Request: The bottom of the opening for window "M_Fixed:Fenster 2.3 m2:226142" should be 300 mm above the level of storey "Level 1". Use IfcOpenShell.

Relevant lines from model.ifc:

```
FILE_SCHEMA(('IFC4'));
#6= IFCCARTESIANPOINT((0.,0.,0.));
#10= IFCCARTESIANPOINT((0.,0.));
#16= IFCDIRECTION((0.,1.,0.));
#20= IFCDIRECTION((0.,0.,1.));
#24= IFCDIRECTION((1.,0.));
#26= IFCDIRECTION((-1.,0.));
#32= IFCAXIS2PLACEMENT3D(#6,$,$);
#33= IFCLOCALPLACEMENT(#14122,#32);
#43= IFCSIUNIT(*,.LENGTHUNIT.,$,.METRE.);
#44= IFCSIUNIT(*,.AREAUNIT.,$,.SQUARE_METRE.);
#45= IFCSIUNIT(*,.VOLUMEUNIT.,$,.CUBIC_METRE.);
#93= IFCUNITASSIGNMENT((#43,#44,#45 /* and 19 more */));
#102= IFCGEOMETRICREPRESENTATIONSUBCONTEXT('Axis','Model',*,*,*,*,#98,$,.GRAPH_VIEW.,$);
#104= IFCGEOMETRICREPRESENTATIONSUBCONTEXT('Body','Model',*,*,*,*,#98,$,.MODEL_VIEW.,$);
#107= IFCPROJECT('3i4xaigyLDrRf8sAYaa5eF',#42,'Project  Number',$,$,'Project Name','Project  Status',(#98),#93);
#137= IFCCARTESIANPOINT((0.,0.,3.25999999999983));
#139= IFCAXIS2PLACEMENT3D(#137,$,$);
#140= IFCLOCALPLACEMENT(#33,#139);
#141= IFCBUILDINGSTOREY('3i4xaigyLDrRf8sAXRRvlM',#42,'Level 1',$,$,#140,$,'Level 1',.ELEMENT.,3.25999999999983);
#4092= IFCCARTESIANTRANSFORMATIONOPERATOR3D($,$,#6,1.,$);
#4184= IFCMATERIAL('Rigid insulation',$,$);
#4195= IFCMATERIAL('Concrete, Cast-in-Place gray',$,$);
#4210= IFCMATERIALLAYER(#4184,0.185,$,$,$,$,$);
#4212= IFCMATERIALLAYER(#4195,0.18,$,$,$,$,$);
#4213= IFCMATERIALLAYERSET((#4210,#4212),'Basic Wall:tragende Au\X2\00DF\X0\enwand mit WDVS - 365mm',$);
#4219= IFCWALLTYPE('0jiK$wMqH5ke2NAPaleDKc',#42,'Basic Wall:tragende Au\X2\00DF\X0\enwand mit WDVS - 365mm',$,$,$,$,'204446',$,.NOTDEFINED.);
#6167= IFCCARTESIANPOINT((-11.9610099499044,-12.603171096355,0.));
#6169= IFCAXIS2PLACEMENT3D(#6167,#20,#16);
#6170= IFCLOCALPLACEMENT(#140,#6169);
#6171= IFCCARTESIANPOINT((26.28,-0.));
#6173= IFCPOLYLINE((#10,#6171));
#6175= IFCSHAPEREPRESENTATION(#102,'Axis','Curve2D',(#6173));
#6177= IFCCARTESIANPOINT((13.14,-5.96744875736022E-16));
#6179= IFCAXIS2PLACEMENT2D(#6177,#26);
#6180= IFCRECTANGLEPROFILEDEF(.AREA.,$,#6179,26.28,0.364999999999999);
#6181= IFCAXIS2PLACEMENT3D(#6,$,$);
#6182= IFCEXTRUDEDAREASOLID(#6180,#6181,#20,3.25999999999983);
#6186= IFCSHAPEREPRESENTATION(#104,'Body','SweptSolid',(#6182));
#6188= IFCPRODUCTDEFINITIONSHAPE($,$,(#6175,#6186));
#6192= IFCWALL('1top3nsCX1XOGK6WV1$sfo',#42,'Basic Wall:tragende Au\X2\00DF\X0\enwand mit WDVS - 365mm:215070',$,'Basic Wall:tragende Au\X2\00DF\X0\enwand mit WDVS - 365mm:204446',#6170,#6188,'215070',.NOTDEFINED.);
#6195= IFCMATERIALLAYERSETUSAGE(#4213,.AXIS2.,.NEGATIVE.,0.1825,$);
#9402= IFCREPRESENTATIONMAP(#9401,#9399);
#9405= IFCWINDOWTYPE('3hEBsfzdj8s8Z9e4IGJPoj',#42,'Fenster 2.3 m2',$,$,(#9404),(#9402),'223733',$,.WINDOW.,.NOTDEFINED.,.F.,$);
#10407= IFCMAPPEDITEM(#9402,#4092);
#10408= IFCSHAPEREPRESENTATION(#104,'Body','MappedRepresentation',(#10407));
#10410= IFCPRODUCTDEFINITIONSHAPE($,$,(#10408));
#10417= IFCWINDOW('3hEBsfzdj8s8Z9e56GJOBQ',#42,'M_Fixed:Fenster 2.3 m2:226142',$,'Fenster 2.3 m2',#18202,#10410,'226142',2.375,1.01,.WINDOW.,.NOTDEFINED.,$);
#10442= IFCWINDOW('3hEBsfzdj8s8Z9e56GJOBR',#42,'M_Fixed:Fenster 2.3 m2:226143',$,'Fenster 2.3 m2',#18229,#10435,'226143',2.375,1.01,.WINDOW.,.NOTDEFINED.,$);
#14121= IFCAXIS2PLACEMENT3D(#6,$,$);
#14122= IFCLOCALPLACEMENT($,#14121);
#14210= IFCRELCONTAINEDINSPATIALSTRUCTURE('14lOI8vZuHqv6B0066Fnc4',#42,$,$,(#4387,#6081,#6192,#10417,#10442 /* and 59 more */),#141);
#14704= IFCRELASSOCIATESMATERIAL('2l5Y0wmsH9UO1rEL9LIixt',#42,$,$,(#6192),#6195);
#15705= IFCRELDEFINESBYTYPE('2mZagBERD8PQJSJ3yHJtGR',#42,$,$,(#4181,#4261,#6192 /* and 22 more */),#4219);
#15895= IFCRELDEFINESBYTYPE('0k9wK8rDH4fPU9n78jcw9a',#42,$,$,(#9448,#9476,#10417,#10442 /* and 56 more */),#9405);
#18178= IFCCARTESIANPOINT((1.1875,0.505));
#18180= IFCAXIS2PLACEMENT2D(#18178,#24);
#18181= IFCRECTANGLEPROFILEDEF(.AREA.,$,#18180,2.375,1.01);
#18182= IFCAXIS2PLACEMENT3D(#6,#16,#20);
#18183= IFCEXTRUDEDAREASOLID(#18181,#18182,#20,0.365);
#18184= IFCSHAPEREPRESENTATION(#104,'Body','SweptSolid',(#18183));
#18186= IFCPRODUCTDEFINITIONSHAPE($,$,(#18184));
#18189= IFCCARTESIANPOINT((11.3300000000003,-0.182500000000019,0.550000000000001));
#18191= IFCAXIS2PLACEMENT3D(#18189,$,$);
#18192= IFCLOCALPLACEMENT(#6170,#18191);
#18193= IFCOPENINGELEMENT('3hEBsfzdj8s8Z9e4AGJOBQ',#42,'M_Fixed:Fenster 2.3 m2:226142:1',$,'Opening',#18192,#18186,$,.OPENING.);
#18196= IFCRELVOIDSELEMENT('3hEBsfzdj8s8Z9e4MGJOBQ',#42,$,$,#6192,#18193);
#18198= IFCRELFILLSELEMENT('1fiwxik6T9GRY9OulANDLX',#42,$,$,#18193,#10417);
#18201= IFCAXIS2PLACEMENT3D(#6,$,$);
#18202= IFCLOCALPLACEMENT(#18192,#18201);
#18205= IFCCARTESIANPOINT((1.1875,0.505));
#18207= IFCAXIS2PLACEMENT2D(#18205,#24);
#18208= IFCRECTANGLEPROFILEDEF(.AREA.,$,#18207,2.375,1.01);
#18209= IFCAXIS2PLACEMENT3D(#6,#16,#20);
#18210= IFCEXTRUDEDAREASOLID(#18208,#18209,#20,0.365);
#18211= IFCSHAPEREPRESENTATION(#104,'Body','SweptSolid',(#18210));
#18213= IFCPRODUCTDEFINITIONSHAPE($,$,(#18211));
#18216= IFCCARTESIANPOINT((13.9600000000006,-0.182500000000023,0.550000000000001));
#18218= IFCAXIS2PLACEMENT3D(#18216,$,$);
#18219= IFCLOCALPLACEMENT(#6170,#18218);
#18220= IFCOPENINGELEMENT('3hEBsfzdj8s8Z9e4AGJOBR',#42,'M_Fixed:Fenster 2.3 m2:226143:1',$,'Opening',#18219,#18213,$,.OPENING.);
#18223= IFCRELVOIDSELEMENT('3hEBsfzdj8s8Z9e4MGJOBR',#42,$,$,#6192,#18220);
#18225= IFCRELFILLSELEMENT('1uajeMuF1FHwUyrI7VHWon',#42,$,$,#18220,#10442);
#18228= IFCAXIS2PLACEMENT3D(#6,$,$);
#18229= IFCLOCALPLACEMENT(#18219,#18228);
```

```python
import numpy as np
import ifcopenshell
import ifcopenshell.api.geometry
import ifcopenshell.geom
import ifcopenshell.util.element
import ifcopenshell.util.placement
import ifcopenshell.util.shape
import ifcopenshell.util.unit

model = ifcopenshell.open("model.ifc")
unit_scale = ifcopenshell.util.unit.calculate_unit_scale(model)

window = model.by_guid("3hEBsfzdj8s8Z9e56GJOBQ")
opening = window.FillsVoids[0].RelatingOpeningElement
storey = ifcopenshell.util.element.get_container(window, ifc_class="IfcBuildingStorey")
level = ifcopenshell.util.placement.get_local_placement(storey.ObjectPlacement)[2, 3]

# The opening's origin need not be at the sill, so measure its lowest point.
shape = ifcopenshell.geom.create_shape(ifcopenshell.geom.settings(), opening)
bottom = ifcopenshell.util.shape.get_shape_bottom_elevation(shape, shape.geometry) / unit_scale
dz = level + 0.3 / unit_scale - bottom

shift = np.array([0.0, 0.0, dz])
# The window is placed relative to its opening, so it follows when the opening moves.
matrix = ifcopenshell.util.placement.get_local_placement(opening.ObjectPlacement)
matrix[:3, 3] += shift
ifcopenshell.api.geometry.edit_object_placement(
    model, product=opening, matrix=matrix, is_si=False, should_transform_children=True
)

print(f"moved by {dz * unit_scale:+.3f} m")

model.write("model_v2.ifc")
```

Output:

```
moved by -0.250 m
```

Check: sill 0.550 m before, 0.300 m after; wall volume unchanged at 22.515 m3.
